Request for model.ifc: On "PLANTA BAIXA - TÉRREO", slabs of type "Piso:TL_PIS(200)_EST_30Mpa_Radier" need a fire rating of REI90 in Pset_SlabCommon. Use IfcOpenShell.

First a look at what the model holds.

```python
import ifcopenshell
import ifcopenshell.util.element

model = ifcopenshell.open("model.ifc")
print(model.schema)
storey = next(s for s in model.by_type("IfcBuildingStorey") if s.Name == "PLANTA BAIXA - TÉRREO")
slabs = [e for e in ifcopenshell.util.element.get_decomposition(storey) if e.is_a("IfcSlab")]
seen = {}
for e in slabs:
    element_type = ifcopenshell.util.element.get_type(e)
    key = (element_type.Name if element_type != e and element_type else None, ifcopenshell.util.element.get_pset(e, "Pset_SlabCommon", "FireRating"))
    seen[key] = seen.get(key, 0) + 1
for (name, value), count in sorted(seen.items(), key=str):
    print(count, "x", name, "|", value)
```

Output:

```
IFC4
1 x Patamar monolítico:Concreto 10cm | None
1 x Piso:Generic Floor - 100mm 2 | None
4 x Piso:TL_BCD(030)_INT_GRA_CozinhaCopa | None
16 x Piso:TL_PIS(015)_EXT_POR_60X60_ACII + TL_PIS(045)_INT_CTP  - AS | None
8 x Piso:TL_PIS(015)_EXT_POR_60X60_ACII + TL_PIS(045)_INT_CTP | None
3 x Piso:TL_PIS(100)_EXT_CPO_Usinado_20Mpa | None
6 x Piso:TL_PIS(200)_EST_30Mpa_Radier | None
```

```python
import ifcopenshell
import ifcopenshell.api.pset
import ifcopenshell.util.element

model = ifcopenshell.open("model.ifc")

storey = next(s for s in model.by_type("IfcBuildingStorey") if s.Name == "PLANTA BAIXA - TÉRREO")
slabs = [e for e in ifcopenshell.util.element.get_decomposition(storey) if e.is_a("IfcSlab")]

count = 0
for e in slabs:
    element_type = ifcopenshell.util.element.get_type(e)
    if element_type in (None, e) or element_type.Name != "Piso:TL_PIS(200)_EST_30Mpa_Radier":
        continue
    # add_pset returns the element's existing set when there is one.
    pset = ifcopenshell.api.pset.add_pset(model, product=e, name="Pset_SlabCommon")
    ifcopenshell.api.pset.edit_pset(model, pset=pset, properties={"FireRating": "REI90"})
    count += 1

print(count, "slabs updated")

model.write("model-out.ifc")
```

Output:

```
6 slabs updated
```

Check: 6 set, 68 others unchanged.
